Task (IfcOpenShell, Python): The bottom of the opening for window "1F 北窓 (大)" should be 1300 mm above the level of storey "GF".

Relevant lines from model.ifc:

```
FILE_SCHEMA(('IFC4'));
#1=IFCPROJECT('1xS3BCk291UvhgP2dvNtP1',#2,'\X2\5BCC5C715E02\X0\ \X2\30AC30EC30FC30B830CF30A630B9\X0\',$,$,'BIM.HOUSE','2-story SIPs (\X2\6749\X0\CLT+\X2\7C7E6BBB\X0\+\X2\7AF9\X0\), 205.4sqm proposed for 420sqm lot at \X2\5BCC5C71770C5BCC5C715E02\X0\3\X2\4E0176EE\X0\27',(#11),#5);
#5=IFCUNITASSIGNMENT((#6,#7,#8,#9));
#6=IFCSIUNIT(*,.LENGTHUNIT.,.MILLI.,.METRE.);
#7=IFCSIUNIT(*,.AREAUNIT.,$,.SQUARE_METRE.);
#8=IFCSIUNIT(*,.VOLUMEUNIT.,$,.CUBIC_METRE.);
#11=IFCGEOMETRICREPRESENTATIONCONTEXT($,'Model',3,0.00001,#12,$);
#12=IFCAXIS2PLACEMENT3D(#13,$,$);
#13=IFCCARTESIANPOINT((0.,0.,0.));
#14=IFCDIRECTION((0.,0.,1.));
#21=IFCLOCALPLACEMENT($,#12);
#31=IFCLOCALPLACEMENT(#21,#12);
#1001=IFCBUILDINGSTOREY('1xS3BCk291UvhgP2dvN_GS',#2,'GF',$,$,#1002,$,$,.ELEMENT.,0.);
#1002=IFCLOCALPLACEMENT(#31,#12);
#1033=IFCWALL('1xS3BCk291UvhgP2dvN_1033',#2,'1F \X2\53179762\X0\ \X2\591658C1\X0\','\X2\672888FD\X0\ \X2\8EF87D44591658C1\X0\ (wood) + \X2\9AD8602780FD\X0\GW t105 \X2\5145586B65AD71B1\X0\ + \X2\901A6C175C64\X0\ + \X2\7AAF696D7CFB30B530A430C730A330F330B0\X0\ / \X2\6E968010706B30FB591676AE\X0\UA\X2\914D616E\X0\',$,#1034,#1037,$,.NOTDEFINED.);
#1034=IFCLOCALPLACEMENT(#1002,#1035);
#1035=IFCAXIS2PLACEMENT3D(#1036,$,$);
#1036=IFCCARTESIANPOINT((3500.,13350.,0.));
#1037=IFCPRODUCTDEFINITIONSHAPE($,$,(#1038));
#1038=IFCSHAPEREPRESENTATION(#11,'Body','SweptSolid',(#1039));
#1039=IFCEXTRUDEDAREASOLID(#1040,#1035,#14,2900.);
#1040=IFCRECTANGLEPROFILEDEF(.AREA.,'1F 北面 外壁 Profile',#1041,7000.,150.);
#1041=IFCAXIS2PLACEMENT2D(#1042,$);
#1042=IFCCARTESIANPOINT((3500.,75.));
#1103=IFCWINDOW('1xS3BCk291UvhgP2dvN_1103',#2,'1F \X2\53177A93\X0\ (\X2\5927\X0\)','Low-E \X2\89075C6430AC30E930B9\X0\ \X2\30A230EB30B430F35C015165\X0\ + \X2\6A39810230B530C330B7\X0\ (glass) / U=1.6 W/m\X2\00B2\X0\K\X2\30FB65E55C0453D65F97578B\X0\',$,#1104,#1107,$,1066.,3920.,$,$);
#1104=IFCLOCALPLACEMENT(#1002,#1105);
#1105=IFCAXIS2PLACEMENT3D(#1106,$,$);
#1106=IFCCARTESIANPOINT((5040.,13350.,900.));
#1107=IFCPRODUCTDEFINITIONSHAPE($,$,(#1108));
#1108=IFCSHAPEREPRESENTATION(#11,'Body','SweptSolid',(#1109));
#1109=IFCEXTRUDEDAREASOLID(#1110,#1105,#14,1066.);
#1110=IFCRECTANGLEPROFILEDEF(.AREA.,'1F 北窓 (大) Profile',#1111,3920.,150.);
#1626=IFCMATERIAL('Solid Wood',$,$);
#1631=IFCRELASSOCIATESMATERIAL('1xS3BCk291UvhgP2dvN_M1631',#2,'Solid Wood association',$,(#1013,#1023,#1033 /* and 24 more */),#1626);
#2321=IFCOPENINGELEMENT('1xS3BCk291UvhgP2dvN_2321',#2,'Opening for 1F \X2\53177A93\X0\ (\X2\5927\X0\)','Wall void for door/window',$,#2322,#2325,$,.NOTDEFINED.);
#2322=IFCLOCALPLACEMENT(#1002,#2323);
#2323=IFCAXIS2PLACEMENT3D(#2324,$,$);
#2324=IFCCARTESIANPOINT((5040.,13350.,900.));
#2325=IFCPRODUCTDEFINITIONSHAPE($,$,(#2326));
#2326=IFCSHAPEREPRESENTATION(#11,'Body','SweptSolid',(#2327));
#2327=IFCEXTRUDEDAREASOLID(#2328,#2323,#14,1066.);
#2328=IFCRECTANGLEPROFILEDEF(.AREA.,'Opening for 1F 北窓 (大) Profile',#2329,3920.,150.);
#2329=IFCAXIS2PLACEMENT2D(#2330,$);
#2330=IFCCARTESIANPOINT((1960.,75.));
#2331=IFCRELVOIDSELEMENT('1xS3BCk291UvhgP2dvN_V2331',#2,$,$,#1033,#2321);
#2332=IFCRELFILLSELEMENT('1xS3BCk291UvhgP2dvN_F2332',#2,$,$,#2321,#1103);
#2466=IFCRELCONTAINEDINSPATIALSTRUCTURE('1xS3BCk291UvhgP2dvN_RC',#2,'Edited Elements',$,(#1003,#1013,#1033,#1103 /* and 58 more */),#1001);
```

```python
import numpy as np
import ifcopenshell
import ifcopenshell.api.geometry
import ifcopenshell.geom
import ifcopenshell.util.element
import ifcopenshell.util.placement
import ifcopenshell.util.shape
import ifcopenshell.util.unit

model = ifcopenshell.open("model.ifc")
unit_scale = ifcopenshell.util.unit.calculate_unit_scale(model)

window = model.by_guid("1xS3BCk291UvhgP2dvN_1103")
opening = window.FillsVoids[0].RelatingOpeningElement
storey = ifcopenshell.util.element.get_container(window, ifc_class="IfcBuildingStorey")
level = ifcopenshell.util.placement.get_local_placement(storey.ObjectPlacement)[2, 3]

# The opening's origin need not be at the sill, so measure its lowest point.
shape = ifcopenshell.geom.create_shape(ifcopenshell.geom.settings(), opening)
bottom = ifcopenshell.util.shape.get_shape_bottom_elevation(shape, shape.geometry) / unit_scale
dz = level + 1.3 / unit_scale - bottom

shift = np.array([0.0, 0.0, dz])
# The window is not placed relative to its opening, so move both.
for product in (opening, window):
    matrix = ifcopenshell.util.placement.get_local_placement(product.ObjectPlacement)
    matrix[:3, 3] += shift
    ifcopenshell.api.geometry.edit_object_placement(model, product=product, matrix=matrix, is_si=False)

print(f"moved by {dz * unit_scale:+.3f} m")

model.write("model_edited.ifc")
```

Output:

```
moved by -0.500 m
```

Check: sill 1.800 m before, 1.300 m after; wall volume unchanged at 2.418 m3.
